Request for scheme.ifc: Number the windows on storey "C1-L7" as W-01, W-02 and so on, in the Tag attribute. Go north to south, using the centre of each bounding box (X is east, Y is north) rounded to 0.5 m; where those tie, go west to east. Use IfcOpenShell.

First a look at what the model holds.

```python
import ifcopenshell
import ifcopenshell.util.element
import ifcopenshell.util.placement

model = ifcopenshell.open("scheme.ifc")
print(model.schema)
storey = next(s for s in model.by_type("IfcBuildingStorey") if s.Name == "C1-L7")
windows = [e for e in ifcopenshell.util.element.get_decomposition(storey) if e.is_a("IfcWindow")]
for e in sorted(windows, key=lambda e: e.id()):
    origin = ifcopenshell.util.placement.get_local_placement(e.ObjectPlacement)[:3, 3]
    print(e.id(), e.Tag, e.Name, origin.round(2) + 0.0, sep=" | ")
```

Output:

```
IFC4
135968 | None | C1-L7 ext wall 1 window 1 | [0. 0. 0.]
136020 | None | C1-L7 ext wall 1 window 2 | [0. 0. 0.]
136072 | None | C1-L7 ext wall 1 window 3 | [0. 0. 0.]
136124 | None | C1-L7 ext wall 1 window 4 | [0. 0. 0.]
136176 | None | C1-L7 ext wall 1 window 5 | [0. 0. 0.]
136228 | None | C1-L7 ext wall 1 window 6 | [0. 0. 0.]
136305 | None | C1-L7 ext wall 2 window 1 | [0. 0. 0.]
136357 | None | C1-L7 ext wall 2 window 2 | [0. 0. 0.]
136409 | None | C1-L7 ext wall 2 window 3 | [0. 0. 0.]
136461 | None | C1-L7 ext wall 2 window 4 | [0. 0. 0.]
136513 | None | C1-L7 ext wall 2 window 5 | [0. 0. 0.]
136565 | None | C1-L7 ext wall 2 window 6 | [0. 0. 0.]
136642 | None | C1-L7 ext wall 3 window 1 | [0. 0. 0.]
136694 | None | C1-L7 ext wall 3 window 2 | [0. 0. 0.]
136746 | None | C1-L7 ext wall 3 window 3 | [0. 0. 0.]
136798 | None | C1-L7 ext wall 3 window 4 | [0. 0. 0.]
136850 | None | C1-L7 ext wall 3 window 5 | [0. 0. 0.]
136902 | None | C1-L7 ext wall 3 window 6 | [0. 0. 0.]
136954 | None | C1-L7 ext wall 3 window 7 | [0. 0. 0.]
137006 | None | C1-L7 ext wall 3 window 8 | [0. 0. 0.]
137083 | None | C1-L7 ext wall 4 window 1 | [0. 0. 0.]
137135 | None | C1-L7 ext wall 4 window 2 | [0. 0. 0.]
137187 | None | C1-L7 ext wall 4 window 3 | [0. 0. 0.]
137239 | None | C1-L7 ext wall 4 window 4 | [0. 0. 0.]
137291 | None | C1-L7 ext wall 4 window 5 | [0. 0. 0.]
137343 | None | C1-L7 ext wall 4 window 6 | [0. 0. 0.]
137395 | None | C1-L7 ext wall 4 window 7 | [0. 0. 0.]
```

```python
import ifcopenshell
import ifcopenshell.geom
import ifcopenshell.util.element
import ifcopenshell.util.shape

model = ifcopenshell.open("scheme.ifc")
settings = ifcopenshell.geom.settings()
settings.set("use-world-coords", True)


def centre(element):
    shape = ifcopenshell.geom.create_shape(settings, element)
    return ifcopenshell.util.shape.get_bbox_centroid(shape.geometry)


storey = next(s for s in model.by_type("IfcBuildingStorey") if s.Name == "C1-L7")
windows = [e for e in ifcopenshell.util.element.get_decomposition(storey) if e.is_a("IfcWindow")]

# Insertion points can sit at a corner or the storey origin, so sort by the geometry (in metres).
centres = {e: centre(e) for e in windows}
windows.sort(key=lambda e: (-round(centres[e][1] / 0.5), centres[e][0]))

for i, e in enumerate(windows, start=1):
    number = f"W-{i:02d}"
    e.Tag = number
    print(e.id(), number)

model.write("scheme_rev.ifc")
```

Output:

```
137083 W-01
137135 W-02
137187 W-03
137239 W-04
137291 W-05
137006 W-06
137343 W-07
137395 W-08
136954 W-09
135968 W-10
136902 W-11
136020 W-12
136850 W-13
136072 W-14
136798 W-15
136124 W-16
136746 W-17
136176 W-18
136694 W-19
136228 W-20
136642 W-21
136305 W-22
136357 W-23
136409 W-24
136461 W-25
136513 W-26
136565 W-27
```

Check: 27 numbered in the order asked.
